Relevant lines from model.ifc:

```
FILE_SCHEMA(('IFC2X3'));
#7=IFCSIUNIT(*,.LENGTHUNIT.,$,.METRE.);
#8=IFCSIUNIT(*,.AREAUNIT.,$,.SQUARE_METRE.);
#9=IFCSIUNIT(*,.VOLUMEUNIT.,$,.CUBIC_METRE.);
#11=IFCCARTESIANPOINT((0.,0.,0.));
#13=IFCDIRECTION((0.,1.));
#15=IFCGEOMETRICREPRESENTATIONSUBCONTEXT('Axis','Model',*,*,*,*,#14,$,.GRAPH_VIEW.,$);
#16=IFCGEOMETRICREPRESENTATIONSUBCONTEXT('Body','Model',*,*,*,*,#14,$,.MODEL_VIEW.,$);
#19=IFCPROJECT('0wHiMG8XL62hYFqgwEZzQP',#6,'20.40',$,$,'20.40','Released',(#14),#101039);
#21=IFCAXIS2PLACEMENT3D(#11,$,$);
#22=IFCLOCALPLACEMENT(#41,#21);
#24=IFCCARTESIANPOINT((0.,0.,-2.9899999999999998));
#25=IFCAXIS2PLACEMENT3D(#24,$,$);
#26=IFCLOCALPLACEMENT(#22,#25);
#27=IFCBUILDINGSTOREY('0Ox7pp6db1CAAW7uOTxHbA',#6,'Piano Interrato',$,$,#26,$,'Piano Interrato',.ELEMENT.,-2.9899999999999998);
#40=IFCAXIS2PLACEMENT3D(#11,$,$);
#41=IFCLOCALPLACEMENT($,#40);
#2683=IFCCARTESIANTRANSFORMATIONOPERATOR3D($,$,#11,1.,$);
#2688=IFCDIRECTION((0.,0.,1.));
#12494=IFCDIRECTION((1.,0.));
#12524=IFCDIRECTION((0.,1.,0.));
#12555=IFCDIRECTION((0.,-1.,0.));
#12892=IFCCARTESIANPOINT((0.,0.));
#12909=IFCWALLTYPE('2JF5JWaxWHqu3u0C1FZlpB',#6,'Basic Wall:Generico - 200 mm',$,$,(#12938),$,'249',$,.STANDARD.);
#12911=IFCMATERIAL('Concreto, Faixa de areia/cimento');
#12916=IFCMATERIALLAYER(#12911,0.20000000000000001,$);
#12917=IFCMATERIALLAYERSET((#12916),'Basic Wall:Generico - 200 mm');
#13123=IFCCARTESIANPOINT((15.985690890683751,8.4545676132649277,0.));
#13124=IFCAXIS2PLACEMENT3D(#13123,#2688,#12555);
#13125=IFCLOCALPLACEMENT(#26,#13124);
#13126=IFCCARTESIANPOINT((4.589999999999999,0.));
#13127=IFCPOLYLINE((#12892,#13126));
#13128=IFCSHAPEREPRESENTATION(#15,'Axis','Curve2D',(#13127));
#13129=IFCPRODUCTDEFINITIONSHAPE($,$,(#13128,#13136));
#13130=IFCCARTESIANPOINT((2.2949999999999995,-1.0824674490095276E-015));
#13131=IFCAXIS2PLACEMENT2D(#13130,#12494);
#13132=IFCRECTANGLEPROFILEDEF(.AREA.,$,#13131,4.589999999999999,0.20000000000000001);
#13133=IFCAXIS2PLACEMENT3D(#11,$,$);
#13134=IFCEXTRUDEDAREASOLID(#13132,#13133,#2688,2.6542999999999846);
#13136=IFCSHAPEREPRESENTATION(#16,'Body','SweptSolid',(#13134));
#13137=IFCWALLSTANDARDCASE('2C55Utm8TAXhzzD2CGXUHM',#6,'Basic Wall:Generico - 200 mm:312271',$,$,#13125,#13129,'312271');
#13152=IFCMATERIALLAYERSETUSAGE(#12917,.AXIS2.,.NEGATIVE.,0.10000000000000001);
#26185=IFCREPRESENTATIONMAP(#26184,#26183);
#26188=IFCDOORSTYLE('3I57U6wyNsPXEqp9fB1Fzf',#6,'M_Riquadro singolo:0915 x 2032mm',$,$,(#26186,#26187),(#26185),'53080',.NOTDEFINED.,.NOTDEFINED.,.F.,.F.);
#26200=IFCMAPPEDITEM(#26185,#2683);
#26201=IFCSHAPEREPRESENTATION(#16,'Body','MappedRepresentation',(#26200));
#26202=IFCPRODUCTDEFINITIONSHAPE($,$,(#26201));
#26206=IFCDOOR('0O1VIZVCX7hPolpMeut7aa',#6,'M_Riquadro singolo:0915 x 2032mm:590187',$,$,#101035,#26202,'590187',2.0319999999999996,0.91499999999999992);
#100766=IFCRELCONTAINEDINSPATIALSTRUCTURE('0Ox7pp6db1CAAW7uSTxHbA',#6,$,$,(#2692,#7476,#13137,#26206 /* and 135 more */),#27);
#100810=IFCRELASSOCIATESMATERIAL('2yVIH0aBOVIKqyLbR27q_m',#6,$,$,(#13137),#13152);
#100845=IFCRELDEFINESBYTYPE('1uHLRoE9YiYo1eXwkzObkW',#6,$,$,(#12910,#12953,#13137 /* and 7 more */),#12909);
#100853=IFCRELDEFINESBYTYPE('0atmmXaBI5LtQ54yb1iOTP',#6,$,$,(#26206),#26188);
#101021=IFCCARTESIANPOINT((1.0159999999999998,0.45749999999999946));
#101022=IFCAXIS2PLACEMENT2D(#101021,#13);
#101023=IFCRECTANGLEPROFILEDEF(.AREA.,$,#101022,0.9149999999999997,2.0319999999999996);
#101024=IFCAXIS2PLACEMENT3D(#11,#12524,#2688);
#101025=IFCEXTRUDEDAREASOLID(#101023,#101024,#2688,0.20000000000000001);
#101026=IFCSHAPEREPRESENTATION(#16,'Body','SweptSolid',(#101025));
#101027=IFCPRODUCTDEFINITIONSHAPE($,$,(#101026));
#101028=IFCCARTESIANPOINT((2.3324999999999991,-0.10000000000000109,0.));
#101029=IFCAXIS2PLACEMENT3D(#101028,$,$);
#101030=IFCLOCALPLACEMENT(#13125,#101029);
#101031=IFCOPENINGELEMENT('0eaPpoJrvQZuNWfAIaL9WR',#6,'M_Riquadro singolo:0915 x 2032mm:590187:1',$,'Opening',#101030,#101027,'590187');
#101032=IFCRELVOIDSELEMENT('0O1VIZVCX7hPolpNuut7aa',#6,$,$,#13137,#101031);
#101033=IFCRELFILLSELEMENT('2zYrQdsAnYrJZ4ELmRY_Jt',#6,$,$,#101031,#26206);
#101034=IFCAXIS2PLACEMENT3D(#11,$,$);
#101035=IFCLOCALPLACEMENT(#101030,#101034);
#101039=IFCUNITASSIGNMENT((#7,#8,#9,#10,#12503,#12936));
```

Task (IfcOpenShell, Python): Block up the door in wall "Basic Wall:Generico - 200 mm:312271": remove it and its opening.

```python
import ifcopenshell
import ifcopenshell.api.feature
import ifcopenshell.api.root
import ifcopenshell.geom
import ifcopenshell.util.shape

model = ifcopenshell.open("model.ifc")
settings = ifcopenshell.geom.settings()


def volume(element):
    """Net volume in cubic metres, openings subtracted."""
    shape = ifcopenshell.geom.create_shape(settings, element)
    return ifcopenshell.util.shape.get_volume(shape.geometry)


door = model.by_guid("0O1VIZVCX7hPolpMeut7aa")
opening = door.FillsVoids[0].RelatingOpeningElement
wall = opening.VoidsElements[0].RelatingBuildingElement
before = volume(wall)

ifcopenshell.api.root.remove_product(model, product=door)
ifcopenshell.api.feature.remove_feature(model, feature=opening)

after = volume(wall)

print(f"wall volume {before:.3f} -> {after:.3f} m3")

model.write("model_v2.ifc")
```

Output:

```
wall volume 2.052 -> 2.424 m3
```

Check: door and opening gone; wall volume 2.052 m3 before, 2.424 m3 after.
